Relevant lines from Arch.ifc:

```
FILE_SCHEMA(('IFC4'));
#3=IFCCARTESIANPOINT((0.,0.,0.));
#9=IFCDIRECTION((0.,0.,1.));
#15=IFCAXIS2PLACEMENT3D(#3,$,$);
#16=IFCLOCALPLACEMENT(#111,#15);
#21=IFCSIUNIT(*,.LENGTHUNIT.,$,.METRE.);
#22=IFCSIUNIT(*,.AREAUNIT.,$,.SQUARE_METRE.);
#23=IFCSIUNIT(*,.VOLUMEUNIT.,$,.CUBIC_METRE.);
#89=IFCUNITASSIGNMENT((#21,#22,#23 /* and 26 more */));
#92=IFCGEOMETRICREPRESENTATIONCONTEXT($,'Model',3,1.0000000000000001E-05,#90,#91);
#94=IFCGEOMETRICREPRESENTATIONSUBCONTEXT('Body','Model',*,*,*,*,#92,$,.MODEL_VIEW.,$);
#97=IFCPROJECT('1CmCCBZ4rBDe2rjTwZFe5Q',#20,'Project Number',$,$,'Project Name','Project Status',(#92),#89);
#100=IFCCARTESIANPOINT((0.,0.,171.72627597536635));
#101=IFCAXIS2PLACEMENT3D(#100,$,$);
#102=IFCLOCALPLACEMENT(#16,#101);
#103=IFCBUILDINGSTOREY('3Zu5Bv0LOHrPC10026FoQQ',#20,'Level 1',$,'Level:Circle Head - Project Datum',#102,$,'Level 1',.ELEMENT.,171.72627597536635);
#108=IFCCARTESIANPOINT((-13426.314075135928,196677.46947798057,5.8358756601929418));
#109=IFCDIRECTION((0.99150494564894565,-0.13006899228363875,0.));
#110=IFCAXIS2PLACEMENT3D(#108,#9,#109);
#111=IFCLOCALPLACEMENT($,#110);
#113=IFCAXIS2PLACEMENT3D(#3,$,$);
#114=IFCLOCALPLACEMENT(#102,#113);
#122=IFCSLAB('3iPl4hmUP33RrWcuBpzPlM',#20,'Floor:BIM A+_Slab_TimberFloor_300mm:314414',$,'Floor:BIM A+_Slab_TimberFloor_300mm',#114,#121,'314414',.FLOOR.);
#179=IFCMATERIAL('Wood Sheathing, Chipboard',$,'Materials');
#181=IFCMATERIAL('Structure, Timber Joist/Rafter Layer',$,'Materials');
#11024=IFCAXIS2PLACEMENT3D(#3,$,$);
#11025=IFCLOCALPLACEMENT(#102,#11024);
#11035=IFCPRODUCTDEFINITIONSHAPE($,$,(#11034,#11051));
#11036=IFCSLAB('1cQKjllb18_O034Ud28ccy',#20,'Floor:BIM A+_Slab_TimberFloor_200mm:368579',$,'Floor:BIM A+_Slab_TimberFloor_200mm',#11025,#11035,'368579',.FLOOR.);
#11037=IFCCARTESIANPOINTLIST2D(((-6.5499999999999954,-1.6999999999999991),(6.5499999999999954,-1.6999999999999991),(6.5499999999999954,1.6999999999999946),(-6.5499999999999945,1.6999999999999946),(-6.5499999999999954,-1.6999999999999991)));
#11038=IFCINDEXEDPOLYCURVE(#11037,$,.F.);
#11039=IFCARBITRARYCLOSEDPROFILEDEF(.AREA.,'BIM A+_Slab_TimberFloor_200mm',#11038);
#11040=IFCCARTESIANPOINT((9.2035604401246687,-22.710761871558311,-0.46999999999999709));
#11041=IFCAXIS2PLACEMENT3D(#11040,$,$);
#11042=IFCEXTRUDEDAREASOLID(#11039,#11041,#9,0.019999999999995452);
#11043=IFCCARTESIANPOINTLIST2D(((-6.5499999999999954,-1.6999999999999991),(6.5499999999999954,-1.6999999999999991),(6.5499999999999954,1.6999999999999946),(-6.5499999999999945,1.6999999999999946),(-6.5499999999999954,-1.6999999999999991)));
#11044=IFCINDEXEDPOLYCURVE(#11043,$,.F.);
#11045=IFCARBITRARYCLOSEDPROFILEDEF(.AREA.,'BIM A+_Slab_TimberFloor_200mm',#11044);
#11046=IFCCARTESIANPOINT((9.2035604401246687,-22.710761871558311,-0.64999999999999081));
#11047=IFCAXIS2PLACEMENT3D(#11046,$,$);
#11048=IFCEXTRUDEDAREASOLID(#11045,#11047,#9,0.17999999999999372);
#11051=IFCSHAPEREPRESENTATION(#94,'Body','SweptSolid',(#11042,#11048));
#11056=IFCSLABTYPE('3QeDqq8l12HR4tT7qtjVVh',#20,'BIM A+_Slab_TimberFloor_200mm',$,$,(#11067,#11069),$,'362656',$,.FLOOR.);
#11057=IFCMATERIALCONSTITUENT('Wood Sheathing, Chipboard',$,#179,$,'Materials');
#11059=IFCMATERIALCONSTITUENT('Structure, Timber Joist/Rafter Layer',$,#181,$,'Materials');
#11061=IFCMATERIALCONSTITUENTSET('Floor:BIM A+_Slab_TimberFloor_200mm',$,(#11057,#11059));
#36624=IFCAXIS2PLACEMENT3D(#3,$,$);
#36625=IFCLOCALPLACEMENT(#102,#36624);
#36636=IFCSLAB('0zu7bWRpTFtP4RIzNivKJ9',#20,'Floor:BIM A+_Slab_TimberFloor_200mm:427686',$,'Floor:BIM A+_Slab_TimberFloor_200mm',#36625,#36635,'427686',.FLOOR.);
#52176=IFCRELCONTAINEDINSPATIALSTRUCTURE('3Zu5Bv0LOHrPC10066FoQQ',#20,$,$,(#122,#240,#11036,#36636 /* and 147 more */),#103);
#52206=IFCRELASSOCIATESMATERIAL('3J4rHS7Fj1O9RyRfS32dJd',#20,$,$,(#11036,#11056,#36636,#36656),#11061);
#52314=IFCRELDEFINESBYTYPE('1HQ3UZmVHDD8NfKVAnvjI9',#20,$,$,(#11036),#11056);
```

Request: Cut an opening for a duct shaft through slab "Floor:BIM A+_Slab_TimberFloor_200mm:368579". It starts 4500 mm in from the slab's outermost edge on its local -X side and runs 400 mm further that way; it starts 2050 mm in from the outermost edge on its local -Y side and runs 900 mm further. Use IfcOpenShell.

```python
import numpy as np
import ifcopenshell
import ifcopenshell.api.feature
import ifcopenshell.api.geometry
import ifcopenshell.api.root
import ifcopenshell.geom
import ifcopenshell.util.placement
import ifcopenshell.util.representation
import ifcopenshell.util.shape
import ifcopenshell.util.unit

model = ifcopenshell.open("Arch.ifc")
unit_scale = ifcopenshell.util.unit.calculate_unit_scale(model)
settings = ifcopenshell.geom.settings()


def volume(element):
    """Net volume in cubic metres, openings subtracted."""
    shape = ifcopenshell.geom.create_shape(settings, element)
    return ifcopenshell.util.shape.get_volume(shape.geometry)


slab = model.by_guid("1cQKjllb18_O034Ud28ccy")
before = volume(slab)

# Extent in the slab's own axes, in metres. The edges named are its -X and -Y sides.
slab_shape = ifcopenshell.geom.create_shape(settings, slab)
vertices = ifcopenshell.util.shape.get_vertices(slab_shape.geometry)
x_min, y_min, bottom = vertices.min(axis=0)
top = vertices[:, 2].max()

opening = ifcopenshell.api.root.create_entity(model, ifc_class="IfcOpeningElement", name="Duct shaft opening", predefined_type="OPENING")
context = ifcopenshell.util.representation.get_context(model, "Model", "Body", "MODEL_VIEW")
width, depth = 0.4, 0.9
outline = [(0.0, 0.0), (width, 0.0), (width, depth), (0.0, depth), (0.0, 0.0)]
# Overshoot both faces by 50 mm so the cut is clean.
shape = ifcopenshell.api.geometry.add_slab_representation(
    model, context=context, depth=top - bottom + 0.1, polyline=outline
)
ifcopenshell.api.geometry.assign_representation(model, product=opening, representation=shape)

matrix = ifcopenshell.util.placement.get_local_placement(slab.ObjectPlacement)
matrix[:, 3] = matrix @ np.append(np.array([x_min + 4.5, y_min + 2.05, bottom - 0.05]) / unit_scale, 1.0)
ifcopenshell.api.geometry.edit_object_placement(model, product=opening, matrix=matrix, is_si=False)
ifcopenshell.api.feature.add_feature(model, feature=opening, element=slab)

after = volume(slab)

print(f"slab volume {before:.3f} -> {after:.3f} m3")

model.write("Arch_edited.ifc")
```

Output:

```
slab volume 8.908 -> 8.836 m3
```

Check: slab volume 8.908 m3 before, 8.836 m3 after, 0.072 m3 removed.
